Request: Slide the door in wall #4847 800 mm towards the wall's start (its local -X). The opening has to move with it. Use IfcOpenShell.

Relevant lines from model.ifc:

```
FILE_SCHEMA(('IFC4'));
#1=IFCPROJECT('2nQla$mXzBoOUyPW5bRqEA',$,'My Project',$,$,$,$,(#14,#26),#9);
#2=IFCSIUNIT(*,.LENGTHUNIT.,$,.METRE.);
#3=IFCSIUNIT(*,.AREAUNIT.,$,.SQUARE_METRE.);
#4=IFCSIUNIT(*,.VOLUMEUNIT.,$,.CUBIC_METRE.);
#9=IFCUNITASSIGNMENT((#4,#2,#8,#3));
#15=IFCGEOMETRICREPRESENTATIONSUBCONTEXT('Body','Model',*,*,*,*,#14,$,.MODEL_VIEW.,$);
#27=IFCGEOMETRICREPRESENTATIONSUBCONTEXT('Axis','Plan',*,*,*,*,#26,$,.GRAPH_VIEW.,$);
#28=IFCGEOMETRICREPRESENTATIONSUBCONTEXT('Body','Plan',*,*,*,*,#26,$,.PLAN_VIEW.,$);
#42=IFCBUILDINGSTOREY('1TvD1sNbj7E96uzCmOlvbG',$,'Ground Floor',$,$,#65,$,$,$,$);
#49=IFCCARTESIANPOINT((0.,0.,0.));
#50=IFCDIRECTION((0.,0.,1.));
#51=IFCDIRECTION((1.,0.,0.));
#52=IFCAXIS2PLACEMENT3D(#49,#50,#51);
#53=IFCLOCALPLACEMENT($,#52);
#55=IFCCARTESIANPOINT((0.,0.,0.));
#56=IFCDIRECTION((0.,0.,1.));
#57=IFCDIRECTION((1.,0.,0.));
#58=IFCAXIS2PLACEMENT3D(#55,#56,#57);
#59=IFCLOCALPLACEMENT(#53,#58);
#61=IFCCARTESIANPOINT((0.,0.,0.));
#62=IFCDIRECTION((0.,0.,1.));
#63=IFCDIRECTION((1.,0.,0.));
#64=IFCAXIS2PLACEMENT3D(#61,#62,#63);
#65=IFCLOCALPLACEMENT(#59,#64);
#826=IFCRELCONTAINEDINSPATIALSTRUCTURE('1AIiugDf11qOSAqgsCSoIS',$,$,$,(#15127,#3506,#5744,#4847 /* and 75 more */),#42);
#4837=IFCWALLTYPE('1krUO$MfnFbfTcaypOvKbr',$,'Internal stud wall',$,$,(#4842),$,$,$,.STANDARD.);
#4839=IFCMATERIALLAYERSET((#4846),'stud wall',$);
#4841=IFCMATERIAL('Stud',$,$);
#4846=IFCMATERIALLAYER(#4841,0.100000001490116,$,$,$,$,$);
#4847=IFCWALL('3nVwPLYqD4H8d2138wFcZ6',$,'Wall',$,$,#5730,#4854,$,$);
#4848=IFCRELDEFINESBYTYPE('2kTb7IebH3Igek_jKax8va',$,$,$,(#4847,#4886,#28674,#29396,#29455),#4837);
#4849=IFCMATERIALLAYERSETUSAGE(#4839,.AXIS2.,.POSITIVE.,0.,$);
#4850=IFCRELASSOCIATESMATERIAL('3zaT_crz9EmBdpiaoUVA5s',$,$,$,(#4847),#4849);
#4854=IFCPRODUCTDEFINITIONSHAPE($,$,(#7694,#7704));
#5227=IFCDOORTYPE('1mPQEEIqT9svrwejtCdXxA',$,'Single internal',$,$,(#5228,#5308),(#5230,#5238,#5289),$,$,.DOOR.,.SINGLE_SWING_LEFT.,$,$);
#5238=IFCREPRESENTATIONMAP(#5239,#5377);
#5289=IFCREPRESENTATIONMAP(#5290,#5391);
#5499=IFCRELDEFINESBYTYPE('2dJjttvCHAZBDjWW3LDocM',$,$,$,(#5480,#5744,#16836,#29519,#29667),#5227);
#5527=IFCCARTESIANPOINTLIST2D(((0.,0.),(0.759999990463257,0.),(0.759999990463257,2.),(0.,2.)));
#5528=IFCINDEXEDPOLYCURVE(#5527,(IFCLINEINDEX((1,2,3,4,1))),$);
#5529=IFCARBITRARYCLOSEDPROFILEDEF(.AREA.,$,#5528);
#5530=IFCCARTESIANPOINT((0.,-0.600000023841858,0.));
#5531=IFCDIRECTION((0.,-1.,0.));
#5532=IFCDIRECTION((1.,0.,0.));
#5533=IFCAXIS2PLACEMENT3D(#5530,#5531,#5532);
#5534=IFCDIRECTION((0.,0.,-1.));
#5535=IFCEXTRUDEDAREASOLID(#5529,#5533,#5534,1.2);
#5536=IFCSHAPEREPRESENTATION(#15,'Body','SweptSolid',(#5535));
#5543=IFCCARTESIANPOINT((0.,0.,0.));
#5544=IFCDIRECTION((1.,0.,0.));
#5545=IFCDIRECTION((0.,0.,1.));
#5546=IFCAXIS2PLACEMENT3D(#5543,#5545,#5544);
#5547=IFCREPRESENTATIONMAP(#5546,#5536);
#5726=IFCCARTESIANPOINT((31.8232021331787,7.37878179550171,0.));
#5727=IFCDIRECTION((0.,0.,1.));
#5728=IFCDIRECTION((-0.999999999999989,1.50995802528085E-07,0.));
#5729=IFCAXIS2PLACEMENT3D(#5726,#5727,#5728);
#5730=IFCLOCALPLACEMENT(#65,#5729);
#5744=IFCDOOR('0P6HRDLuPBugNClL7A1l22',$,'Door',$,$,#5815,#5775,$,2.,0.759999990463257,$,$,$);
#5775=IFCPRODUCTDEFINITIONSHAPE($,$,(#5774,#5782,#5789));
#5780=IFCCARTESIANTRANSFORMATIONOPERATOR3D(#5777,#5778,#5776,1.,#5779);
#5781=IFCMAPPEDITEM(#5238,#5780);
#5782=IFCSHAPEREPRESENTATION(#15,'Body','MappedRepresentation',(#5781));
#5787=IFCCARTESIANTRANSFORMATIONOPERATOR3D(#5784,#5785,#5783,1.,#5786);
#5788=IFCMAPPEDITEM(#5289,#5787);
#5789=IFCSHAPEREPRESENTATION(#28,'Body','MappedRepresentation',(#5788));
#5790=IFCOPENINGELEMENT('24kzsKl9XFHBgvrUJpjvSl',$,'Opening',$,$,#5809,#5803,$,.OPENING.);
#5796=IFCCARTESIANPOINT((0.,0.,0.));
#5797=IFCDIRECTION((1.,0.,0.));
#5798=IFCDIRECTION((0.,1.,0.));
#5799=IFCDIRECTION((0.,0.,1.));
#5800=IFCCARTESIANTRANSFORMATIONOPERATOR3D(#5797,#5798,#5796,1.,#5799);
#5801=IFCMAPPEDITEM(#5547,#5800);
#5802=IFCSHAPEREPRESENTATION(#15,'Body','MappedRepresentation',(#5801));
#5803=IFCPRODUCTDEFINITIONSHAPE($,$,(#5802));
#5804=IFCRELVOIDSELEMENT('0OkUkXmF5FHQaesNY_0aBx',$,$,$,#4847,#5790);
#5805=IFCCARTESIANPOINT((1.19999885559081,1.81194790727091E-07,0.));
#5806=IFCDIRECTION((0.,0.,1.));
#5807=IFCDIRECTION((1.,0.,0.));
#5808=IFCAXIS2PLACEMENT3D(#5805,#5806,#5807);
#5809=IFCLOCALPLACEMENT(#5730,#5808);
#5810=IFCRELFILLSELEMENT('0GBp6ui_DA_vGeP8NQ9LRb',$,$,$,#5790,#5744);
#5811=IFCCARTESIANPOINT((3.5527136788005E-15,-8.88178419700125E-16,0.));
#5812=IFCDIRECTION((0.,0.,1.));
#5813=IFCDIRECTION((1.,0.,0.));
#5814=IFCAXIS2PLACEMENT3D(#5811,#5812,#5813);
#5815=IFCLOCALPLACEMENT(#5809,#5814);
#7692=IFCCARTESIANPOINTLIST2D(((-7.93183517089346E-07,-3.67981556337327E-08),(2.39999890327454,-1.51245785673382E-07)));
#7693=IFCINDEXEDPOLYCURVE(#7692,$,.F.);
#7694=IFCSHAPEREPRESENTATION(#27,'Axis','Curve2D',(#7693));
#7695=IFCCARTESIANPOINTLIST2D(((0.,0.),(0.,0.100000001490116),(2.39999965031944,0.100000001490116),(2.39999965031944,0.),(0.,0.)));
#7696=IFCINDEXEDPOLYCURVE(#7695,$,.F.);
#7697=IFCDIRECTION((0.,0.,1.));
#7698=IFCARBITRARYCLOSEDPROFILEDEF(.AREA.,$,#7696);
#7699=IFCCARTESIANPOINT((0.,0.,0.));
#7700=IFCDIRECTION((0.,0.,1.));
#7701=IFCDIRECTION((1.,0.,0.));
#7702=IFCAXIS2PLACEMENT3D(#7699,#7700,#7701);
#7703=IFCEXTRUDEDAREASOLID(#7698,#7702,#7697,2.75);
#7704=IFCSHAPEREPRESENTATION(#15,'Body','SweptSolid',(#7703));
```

```python
import ifcopenshell
import ifcopenshell.api.geometry
import ifcopenshell.util.placement
import ifcopenshell.util.unit

model = ifcopenshell.open("model.ifc")
unit_scale = ifcopenshell.util.unit.calculate_unit_scale(model)

door = model.by_guid("0P6HRDLuPBugNClL7A1l22")
opening = door.FillsVoids[0].RelatingOpeningElement
wall = opening.VoidsElements[0].RelatingBuildingElement

wall_matrix = ifcopenshell.util.placement.get_local_placement(wall.ObjectPlacement)
shift = wall_matrix[:3, 0] * -0.8 / unit_scale
before = ifcopenshell.util.placement.get_local_placement(door.ObjectPlacement)[:3, 3].copy()

# The door is placed relative to its opening, so it follows when the opening moves.
matrix = ifcopenshell.util.placement.get_local_placement(opening.ObjectPlacement)
matrix[:3, 3] += shift
ifcopenshell.api.geometry.edit_object_placement(
    model, product=opening, matrix=matrix, is_si=False, should_transform_children=True
)

after = ifcopenshell.util.placement.get_local_placement(door.ObjectPlacement)[:3, 3]
print("door moved by", (after - before).round(3) + 0.0)

model.write("model_updated.ifc")
```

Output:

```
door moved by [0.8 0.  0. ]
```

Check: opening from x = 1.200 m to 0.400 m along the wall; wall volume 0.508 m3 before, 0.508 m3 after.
